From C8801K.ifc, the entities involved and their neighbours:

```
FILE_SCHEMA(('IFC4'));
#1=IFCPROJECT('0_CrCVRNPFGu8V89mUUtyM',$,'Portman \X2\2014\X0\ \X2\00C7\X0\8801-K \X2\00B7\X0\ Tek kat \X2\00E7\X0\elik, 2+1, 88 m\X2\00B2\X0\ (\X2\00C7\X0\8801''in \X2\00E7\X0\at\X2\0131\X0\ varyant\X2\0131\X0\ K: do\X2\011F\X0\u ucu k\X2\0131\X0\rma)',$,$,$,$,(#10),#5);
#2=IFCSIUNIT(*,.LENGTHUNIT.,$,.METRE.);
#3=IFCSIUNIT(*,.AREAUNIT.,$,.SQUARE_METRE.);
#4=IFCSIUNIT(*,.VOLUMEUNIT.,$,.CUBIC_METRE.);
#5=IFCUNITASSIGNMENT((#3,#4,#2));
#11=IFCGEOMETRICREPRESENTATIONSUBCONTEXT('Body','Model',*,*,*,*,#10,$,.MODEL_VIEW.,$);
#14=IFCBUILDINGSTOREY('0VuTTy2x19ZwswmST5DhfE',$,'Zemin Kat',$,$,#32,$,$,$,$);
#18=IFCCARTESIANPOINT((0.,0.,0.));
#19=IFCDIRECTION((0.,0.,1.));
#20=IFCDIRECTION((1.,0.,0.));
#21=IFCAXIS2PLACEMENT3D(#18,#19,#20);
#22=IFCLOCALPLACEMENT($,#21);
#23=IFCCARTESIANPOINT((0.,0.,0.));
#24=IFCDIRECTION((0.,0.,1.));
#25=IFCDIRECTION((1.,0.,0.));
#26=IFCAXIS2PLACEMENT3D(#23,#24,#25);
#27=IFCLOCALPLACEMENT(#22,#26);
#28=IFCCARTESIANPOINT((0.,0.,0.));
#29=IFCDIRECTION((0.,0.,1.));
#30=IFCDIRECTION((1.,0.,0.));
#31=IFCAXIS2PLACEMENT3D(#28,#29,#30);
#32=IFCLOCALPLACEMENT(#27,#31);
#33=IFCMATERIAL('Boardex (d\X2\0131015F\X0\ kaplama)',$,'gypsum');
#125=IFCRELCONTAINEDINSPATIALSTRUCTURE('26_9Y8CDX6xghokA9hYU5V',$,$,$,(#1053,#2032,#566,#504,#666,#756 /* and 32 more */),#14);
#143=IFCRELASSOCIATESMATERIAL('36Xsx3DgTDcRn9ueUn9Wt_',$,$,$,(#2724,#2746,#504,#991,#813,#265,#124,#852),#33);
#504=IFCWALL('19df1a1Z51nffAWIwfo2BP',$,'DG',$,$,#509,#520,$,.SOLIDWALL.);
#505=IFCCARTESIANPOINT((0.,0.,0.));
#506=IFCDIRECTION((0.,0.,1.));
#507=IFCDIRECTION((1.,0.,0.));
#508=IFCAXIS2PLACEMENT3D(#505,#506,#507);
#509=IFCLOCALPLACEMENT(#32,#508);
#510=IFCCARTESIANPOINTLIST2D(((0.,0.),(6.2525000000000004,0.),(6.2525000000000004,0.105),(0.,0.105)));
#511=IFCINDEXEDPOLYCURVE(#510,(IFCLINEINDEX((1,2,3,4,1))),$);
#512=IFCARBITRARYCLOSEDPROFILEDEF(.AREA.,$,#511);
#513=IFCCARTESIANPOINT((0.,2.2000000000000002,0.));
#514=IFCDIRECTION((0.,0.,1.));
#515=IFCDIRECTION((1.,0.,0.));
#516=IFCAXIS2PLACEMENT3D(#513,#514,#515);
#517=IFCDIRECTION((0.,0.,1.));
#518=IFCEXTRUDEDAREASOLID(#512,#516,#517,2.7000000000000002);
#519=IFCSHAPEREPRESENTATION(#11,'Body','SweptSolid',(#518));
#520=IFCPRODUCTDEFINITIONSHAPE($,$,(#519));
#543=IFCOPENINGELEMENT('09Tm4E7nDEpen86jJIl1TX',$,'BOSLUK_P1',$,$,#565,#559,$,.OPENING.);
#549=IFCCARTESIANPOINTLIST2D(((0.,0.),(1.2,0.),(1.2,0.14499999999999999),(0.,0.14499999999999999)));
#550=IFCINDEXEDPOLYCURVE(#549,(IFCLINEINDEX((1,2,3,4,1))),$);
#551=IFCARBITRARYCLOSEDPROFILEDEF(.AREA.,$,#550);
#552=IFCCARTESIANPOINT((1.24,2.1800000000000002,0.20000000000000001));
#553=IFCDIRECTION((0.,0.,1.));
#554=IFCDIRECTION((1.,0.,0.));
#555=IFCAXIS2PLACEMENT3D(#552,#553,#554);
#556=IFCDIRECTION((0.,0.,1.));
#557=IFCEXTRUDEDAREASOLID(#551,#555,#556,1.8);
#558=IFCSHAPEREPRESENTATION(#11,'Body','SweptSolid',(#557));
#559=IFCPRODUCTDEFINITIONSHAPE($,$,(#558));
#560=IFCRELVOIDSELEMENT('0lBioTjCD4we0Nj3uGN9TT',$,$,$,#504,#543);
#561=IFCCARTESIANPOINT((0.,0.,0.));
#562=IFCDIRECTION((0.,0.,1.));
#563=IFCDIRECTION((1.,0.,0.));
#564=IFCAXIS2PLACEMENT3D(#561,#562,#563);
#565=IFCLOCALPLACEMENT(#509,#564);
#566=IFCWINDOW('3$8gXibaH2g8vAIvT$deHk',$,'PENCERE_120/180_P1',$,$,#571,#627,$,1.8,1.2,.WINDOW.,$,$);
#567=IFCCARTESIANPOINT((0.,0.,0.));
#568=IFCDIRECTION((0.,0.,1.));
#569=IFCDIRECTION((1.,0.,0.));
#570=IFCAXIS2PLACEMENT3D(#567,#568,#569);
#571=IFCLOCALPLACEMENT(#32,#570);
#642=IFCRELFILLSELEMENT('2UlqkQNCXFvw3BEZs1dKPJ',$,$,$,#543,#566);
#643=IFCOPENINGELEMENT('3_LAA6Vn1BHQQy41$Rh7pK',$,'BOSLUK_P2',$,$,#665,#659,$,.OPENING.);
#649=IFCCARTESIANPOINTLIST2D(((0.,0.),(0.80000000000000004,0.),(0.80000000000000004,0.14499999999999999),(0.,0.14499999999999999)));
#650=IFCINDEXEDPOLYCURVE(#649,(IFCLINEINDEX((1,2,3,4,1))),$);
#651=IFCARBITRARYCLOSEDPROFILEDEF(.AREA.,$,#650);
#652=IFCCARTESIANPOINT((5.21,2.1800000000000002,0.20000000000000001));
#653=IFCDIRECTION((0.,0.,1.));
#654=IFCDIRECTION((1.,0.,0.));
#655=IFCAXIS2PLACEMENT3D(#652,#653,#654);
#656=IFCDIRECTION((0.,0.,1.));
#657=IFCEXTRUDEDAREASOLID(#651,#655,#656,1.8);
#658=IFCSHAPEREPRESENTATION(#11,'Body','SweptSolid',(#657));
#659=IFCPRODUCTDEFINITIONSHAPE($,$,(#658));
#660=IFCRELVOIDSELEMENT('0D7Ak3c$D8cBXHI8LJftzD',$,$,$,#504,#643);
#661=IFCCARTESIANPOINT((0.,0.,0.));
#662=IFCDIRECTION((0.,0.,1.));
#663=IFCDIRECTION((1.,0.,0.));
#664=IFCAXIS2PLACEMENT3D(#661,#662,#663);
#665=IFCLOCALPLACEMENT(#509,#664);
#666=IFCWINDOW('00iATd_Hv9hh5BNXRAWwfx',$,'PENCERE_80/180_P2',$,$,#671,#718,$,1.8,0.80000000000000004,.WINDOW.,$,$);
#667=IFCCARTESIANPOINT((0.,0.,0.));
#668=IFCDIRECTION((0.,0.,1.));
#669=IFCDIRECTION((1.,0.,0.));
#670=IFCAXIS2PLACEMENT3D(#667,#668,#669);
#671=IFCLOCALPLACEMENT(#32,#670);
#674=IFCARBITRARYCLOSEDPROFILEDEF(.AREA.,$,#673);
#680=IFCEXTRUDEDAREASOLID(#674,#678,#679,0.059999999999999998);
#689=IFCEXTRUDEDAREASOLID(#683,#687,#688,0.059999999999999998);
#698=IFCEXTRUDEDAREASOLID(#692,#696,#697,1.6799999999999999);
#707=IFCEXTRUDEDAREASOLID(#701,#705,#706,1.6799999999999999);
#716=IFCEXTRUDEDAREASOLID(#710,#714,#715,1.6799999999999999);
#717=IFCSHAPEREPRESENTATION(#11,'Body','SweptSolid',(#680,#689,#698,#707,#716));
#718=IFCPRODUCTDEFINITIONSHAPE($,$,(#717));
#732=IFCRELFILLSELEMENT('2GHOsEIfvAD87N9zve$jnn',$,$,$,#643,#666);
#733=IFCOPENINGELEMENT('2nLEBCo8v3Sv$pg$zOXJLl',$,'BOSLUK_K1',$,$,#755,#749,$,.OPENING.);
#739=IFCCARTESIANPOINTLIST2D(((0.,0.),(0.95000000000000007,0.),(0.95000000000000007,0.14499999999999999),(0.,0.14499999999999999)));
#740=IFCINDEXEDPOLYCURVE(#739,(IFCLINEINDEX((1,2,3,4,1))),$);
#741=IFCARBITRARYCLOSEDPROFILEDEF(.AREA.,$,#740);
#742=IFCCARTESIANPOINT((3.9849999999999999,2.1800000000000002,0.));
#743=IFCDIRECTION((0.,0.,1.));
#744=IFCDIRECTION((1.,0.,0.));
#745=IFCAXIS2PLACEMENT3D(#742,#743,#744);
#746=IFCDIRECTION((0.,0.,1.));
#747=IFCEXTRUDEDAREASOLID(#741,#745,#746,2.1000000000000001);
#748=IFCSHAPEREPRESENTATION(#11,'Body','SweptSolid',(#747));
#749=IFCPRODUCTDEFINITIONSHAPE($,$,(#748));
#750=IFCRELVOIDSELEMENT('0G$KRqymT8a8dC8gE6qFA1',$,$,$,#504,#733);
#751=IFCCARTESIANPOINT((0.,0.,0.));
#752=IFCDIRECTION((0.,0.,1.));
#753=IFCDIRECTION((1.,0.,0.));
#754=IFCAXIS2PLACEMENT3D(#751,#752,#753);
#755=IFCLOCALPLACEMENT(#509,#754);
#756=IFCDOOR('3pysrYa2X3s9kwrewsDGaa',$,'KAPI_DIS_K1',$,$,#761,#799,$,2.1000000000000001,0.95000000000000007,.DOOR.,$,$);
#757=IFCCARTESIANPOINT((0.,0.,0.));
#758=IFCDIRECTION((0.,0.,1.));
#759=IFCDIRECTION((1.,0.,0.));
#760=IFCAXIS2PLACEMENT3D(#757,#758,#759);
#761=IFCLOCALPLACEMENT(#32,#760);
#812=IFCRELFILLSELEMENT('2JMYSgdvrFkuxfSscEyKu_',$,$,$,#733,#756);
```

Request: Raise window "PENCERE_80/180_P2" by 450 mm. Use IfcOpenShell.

```python
import numpy as np
import ifcopenshell
import ifcopenshell.api.geometry
import ifcopenshell.util.placement
import ifcopenshell.util.unit

model = ifcopenshell.open("C8801K.ifc")
unit_scale = ifcopenshell.util.unit.calculate_unit_scale(model)

window = model.by_guid("00iATd_Hv9hh5BNXRAWwfx")
opening = window.FillsVoids[0].RelatingOpeningElement
dz = 0.45 / unit_scale

shift = np.array([0.0, 0.0, dz])
# The window is not placed relative to its opening, so move both.
for product in (opening, window):
    matrix = ifcopenshell.util.placement.get_local_placement(product.ObjectPlacement)
    matrix[:3, 3] += shift
    ifcopenshell.api.geometry.edit_object_placement(model, product=product, matrix=matrix, is_si=False)

print(f"moved by {dz * unit_scale:+.3f} m")

model.write("C8801K_rev.ifc")
```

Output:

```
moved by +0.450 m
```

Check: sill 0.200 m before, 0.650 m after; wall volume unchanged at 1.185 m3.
